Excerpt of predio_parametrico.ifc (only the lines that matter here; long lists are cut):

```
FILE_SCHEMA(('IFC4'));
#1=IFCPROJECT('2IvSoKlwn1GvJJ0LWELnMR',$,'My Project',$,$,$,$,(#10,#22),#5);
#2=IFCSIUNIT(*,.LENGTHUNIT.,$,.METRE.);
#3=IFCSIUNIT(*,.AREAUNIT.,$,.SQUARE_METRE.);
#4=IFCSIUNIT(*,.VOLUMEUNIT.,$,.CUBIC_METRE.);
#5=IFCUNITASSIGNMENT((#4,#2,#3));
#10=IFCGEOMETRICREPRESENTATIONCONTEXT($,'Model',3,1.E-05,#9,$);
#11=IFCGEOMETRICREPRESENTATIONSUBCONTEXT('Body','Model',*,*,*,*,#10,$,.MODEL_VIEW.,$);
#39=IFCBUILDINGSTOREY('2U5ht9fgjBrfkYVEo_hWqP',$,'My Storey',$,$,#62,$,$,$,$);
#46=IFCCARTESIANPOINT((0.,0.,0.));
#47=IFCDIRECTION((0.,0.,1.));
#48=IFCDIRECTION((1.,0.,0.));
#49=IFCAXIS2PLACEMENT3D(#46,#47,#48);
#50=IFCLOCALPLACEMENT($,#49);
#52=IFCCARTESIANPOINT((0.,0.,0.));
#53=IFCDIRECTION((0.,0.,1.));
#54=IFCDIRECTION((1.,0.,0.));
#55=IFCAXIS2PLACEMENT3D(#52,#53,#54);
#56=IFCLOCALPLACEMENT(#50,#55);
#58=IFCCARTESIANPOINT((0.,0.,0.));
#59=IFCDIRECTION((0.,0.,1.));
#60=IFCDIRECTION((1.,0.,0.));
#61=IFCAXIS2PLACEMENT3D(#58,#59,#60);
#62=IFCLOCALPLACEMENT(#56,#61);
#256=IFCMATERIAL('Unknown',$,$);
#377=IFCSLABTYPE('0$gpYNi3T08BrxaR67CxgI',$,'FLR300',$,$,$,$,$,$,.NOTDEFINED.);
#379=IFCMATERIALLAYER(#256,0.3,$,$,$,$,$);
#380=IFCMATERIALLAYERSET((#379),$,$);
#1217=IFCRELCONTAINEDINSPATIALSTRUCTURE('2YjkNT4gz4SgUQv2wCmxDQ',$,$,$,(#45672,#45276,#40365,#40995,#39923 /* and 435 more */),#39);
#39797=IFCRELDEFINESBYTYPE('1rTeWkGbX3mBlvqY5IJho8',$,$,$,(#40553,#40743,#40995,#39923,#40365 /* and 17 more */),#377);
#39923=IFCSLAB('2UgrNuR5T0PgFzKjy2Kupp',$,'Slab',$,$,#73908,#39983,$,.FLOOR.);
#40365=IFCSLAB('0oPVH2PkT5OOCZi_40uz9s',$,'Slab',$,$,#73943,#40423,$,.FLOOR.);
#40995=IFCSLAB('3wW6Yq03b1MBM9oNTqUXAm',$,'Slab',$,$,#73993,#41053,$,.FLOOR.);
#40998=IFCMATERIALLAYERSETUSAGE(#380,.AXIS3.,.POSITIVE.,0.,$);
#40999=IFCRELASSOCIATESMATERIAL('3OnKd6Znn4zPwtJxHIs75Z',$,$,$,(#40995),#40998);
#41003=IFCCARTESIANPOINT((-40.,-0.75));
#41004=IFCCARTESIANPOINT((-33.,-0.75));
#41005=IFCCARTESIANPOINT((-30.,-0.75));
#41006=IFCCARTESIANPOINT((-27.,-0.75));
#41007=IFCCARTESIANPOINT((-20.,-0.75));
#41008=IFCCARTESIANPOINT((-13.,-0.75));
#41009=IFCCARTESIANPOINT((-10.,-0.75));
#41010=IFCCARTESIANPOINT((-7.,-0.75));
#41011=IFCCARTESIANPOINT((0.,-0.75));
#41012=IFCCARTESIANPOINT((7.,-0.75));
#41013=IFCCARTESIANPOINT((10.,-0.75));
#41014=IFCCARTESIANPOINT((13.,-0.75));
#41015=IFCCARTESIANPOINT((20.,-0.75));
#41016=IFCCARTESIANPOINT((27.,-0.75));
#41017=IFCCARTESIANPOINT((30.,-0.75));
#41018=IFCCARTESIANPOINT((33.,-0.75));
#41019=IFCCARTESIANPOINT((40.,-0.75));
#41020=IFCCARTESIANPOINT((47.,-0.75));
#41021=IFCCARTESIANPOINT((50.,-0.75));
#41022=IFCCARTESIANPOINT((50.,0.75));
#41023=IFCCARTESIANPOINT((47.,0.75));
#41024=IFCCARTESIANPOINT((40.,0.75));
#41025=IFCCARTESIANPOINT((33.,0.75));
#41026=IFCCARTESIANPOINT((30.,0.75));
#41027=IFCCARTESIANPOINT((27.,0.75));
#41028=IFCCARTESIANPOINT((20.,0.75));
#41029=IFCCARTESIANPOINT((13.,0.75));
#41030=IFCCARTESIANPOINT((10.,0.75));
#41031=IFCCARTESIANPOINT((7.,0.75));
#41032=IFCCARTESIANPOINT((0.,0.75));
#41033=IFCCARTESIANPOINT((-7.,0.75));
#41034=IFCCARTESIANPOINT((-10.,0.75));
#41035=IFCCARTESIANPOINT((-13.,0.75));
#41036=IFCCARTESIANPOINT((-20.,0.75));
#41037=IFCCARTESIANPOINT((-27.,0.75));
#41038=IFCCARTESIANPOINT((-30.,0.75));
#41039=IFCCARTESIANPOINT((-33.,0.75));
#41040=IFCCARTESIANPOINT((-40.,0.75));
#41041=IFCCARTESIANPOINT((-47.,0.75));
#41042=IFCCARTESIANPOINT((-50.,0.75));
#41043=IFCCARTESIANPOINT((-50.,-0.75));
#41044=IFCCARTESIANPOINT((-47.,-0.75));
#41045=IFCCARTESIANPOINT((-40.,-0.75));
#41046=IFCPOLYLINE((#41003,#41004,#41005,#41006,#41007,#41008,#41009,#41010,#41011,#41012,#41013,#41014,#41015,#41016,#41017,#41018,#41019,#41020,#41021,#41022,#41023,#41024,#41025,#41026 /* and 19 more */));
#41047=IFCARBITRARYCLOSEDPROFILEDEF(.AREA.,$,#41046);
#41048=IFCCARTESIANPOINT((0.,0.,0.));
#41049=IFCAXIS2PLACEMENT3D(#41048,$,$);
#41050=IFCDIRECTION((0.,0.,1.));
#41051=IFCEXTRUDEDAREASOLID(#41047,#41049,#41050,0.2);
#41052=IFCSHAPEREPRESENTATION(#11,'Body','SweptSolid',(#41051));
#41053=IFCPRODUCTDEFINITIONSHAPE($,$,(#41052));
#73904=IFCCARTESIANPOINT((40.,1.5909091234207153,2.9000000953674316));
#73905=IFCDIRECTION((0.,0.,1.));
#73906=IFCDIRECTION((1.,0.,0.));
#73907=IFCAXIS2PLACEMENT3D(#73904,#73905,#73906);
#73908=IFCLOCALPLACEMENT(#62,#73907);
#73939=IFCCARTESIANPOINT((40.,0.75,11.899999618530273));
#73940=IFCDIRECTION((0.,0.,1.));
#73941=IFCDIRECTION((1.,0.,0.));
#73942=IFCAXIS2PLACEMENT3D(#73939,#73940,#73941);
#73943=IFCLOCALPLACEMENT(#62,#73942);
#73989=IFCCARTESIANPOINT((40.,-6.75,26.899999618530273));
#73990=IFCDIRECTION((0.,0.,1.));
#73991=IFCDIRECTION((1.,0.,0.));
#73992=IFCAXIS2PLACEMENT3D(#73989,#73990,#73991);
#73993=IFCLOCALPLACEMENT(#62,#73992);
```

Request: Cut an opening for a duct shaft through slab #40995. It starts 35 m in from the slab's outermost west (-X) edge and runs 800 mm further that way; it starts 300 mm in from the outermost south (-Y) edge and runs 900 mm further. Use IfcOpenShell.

```python
import numpy as np
import ifcopenshell
import ifcopenshell.api.feature
import ifcopenshell.api.geometry
import ifcopenshell.api.root
import ifcopenshell.geom
import ifcopenshell.util.placement
import ifcopenshell.util.representation
import ifcopenshell.util.shape
import ifcopenshell.util.unit

model = ifcopenshell.open("predio_parametrico.ifc")
unit_scale = ifcopenshell.util.unit.calculate_unit_scale(model)
settings = ifcopenshell.geom.settings()


def volume(element):
    """Net volume in cubic metres, openings subtracted."""
    shape = ifcopenshell.geom.create_shape(settings, element)
    return ifcopenshell.util.shape.get_volume(shape.geometry)


slab = model.by_guid("3wW6Yq03b1MBM9oNTqUXAm")
before = volume(slab)

# Extent in the slab's own axes, in metres. The edges named are its -X and -Y sides.
slab_shape = ifcopenshell.geom.create_shape(settings, slab)
vertices = ifcopenshell.util.shape.get_vertices(slab_shape.geometry)
x_min, y_min, bottom = vertices.min(axis=0)
top = vertices[:, 2].max()

opening = ifcopenshell.api.root.create_entity(model, ifc_class="IfcOpeningElement", name="Duct shaft opening", predefined_type="OPENING")
context = ifcopenshell.util.representation.get_context(model, "Model", "Body", "MODEL_VIEW")
width, depth = 0.8, 0.9
outline = [(0.0, 0.0), (width, 0.0), (width, depth), (0.0, depth), (0.0, 0.0)]
# Overshoot both faces by 50 mm so the cut is clean.
shape = ifcopenshell.api.geometry.add_slab_representation(
    model, context=context, depth=top - bottom + 0.1, polyline=outline
)
ifcopenshell.api.geometry.assign_representation(model, product=opening, representation=shape)

matrix = ifcopenshell.util.placement.get_local_placement(slab.ObjectPlacement)
matrix[:, 3] = matrix @ np.append(np.array([x_min + 35, y_min + 0.3, bottom - 0.05]) / unit_scale, 1.0)
ifcopenshell.api.geometry.edit_object_placement(model, product=opening, matrix=matrix, is_si=False)
ifcopenshell.api.feature.add_feature(model, feature=opening, element=slab)

after = volume(slab)

print(f"slab volume {before:.3f} -> {after:.3f} m3")

model.write("predio_parametrico_updated.ifc")
```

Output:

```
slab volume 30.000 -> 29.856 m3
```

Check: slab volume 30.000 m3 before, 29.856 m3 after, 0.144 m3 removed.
